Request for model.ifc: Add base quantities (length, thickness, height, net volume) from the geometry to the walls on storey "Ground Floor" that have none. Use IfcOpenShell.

First a look at what the model holds.

```python
import ifcopenshell
import ifcopenshell.util.element
import ifcopenshell.util.unit

model = ifcopenshell.open("model.ifc")
print(model.schema)
for unit_type in ("LENGTHUNIT", "AREAUNIT", "VOLUMEUNIT"):
    print(unit_type, ifcopenshell.util.unit.calculate_unit_scale(model, unit_type))
storey = next(s for s in model.by_type("IfcBuildingStorey") if s.Name == "Ground Floor")
walls = [e for e in ifcopenshell.util.element.get_decomposition(storey) if e.is_a("IfcWall")]
for e in sorted(walls, key=lambda e: e.id()):
    print(e.id(), e.is_a(), e.Name, list(ifcopenshell.util.element.get_psets(e, qtos_only=True)), sep=" | ")
```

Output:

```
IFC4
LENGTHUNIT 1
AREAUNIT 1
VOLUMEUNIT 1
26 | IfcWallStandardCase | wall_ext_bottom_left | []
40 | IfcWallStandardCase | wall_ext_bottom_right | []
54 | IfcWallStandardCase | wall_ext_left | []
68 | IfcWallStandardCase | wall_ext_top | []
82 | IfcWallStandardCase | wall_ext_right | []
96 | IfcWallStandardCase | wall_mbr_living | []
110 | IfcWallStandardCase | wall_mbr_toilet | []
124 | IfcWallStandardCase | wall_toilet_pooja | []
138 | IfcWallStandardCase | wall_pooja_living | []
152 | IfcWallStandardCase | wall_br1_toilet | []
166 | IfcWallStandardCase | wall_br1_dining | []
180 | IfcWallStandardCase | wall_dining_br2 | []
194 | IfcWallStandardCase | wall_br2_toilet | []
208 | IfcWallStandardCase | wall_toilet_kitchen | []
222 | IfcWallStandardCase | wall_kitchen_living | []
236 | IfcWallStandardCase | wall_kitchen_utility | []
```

```python
import ifcopenshell
import ifcopenshell.api.pset
import ifcopenshell.geom
import ifcopenshell.util.element
import ifcopenshell.util.shape
import ifcopenshell.util.unit

model = ifcopenshell.open("model.ifc")
unit_scale = ifcopenshell.util.unit.calculate_unit_scale(model)
volume_scale = ifcopenshell.util.unit.calculate_unit_scale(model, "VOLUMEUNIT")
settings = ifcopenshell.geom.settings()

storey = next(s for s in model.by_type("IfcBuildingStorey") if s.Name == "Ground Floor")
walls = [e for e in ifcopenshell.util.element.get_decomposition(storey) if e.is_a("IfcWall")]

for e in sorted(walls, key=lambda e: e.id()):
    if ifcopenshell.util.element.get_psets(e, qtos_only=True, should_inherit=False):
        continue
    # Geometry comes back in metres, in the element's own axes.
    shape = ifcopenshell.geom.create_shape(settings, e)
    values = {
        "Length": ifcopenshell.util.shape.get_x(shape.geometry) / unit_scale,
        "Width": ifcopenshell.util.shape.get_y(shape.geometry) / unit_scale,
        "Height": ifcopenshell.util.shape.get_z(shape.geometry) / unit_scale,
        "NetVolume": ifcopenshell.util.shape.get_volume(shape.geometry) / volume_scale,
    }
    qto = ifcopenshell.api.pset.add_qto(model, product=e, name="Qto_WallBaseQuantities")
    ifcopenshell.api.pset.edit_qto(model, qto=qto, properties=values)
    print(e.id(), {k: round(v, 3) for k, v in values.items()})

model.write("model-out.ifc")
```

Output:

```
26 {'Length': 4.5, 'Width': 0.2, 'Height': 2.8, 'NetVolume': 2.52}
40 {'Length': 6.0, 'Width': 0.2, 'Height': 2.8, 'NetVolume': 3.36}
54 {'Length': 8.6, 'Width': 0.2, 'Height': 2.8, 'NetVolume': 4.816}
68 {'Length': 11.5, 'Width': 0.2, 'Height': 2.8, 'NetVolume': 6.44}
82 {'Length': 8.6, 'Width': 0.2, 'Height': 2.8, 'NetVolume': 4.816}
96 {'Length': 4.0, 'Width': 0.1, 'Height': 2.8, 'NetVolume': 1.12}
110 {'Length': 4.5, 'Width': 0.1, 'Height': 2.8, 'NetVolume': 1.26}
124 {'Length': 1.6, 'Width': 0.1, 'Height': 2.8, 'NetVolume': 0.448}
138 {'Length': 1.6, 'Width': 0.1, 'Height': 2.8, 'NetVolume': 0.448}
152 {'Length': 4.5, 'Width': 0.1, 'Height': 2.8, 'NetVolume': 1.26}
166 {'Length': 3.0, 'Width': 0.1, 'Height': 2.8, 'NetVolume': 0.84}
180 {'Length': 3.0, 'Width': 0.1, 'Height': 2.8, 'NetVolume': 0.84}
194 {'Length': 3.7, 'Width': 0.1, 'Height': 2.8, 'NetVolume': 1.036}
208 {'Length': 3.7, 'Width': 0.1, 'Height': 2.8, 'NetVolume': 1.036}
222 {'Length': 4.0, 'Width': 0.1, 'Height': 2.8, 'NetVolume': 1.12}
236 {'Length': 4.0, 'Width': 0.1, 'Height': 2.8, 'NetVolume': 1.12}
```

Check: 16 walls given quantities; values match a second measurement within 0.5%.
